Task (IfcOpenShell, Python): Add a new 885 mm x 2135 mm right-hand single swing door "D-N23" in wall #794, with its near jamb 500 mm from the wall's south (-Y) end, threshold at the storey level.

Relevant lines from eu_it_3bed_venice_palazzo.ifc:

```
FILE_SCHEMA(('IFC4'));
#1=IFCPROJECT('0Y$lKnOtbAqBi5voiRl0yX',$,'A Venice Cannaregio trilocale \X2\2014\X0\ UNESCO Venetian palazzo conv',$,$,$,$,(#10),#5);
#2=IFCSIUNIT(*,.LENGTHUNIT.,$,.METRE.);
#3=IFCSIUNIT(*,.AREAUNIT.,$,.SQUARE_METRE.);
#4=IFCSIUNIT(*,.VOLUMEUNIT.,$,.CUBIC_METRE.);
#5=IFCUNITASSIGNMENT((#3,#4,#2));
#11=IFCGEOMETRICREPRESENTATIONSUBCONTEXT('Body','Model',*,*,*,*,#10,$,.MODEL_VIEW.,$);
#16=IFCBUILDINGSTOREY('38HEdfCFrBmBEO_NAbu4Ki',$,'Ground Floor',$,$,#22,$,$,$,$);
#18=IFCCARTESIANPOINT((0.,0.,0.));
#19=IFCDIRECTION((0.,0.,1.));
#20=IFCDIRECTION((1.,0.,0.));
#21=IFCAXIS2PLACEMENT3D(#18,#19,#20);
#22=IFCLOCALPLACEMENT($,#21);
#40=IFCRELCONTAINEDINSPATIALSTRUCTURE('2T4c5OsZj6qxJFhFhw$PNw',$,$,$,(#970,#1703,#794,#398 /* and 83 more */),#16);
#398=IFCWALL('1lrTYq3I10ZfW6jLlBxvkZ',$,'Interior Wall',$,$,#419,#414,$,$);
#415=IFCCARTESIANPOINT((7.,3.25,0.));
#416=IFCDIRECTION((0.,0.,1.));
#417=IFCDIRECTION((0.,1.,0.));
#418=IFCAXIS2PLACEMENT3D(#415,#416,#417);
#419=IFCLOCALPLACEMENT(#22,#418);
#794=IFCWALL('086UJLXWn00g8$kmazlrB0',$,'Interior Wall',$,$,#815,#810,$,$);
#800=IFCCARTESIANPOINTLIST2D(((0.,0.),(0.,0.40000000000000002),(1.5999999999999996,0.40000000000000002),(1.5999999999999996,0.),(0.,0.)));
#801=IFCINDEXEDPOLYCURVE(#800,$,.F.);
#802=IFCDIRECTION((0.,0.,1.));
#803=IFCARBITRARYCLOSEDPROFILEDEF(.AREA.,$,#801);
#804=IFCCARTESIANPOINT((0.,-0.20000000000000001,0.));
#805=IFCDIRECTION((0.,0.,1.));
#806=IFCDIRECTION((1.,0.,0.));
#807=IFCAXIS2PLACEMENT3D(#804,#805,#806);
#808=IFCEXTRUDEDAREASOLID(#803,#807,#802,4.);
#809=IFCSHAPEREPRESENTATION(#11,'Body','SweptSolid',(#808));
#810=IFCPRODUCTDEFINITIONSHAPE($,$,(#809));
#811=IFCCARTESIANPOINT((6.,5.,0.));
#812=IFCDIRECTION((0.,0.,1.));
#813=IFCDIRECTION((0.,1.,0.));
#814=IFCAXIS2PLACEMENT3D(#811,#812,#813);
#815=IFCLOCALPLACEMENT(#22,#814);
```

```python
import numpy as np
import ifcopenshell
import ifcopenshell.api.feature
import ifcopenshell.api.geometry
import ifcopenshell.api.root
import ifcopenshell.api.spatial
import ifcopenshell.geom
import ifcopenshell.util.element
import ifcopenshell.util.placement
import ifcopenshell.util.representation
import ifcopenshell.util.shape
import ifcopenshell.util.unit

model = ifcopenshell.open("eu_it_3bed_venice_palazzo.ifc")
unit_scale = ifcopenshell.util.unit.calculate_unit_scale(model)
settings = ifcopenshell.geom.settings()


def volume(element):
    """Net volume in cubic metres, openings subtracted."""
    shape = ifcopenshell.geom.create_shape(settings, element)
    return ifcopenshell.util.shape.get_volume(shape.geometry)


wall = model.by_id(794)
storey = ifcopenshell.util.element.get_container(wall, ifc_class="IfcBuildingStorey")
context = ifcopenshell.util.representation.get_context(model, "Model", "Body", "MODEL_VIEW")
before = volume(wall)

width, height, from_end, sill = 0.885, 2.135, 0.5, 0.0  # metres

# The wall runs along its own X axis, and the end named is its -X end.
wall_shape = ifcopenshell.geom.create_shape(settings, wall)
x, y, z = ifcopenshell.util.shape.get_vertices(wall_shape.geometry).T
start = x.min() + from_end
face, thickness = float(y.min()), float(y.max() - y.min())
wall_matrix = ifcopenshell.util.placement.get_local_placement(wall.ObjectPlacement)
level = ifcopenshell.util.placement.get_local_placement(storey.ObjectPlacement)[2, 3]


def in_wall(x, y):
    """Placement at x, y metres in the wall's axes, at sill height."""
    matrix = wall_matrix.copy()
    matrix[:, 3] = wall_matrix @ np.array([x / unit_scale, y / unit_scale, 0.0, 1.0])
    matrix[2, 3] = level + sill / unit_scale
    return matrix


# Opening: a box that overshoots both wall faces by 50 mm.
opening = ifcopenshell.api.root.create_entity(model, ifc_class="IfcOpeningElement", predefined_type="OPENING")
box = ifcopenshell.api.geometry.add_wall_representation(
    model, context=context, length=width, height=height, thickness=thickness + 0.1
)
ifcopenshell.api.geometry.assign_representation(model, product=opening, representation=box)
ifcopenshell.api.geometry.edit_object_placement(model, product=opening, matrix=in_wall(start, face - 0.05), is_si=False)
ifcopenshell.api.feature.add_feature(model, feature=opening, element=wall)

door = ifcopenshell.api.root.create_entity(model, ifc_class="IfcDoor", name="D-N23", predefined_type="DOOR")
door.OverallWidth, door.OverallHeight = width / unit_scale, height / unit_scale
door.OperationType = "SINGLE_SWING_RIGHT"
body = ifcopenshell.api.geometry.add_door_representation(
    model,
    context=context,
    overall_width=door.OverallWidth,
    overall_height=door.OverallHeight,
    operation_type="SINGLE_SWING_RIGHT",
    lining_properties={"LiningDepth": thickness / unit_scale, "ThresholdDepth": thickness / unit_scale},
)
ifcopenshell.api.geometry.assign_representation(model, product=door, representation=body)
ifcopenshell.api.spatial.assign_container(model, products=[door], relating_structure=storey)
ifcopenshell.api.feature.add_filling(model, opening=opening, element=door)

# The lining spans the wall, so the door starts at the wall face.
ifcopenshell.api.geometry.edit_object_placement(model, product=door, matrix=in_wall(start, face), is_si=False)

after = volume(wall)

print(f"wall volume {before:.3f} -> {after:.3f} m3")

model.write("eu_it_3bed_venice_palazzo_rev.ifc")
```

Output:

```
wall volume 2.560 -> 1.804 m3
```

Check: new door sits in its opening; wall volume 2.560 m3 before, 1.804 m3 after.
